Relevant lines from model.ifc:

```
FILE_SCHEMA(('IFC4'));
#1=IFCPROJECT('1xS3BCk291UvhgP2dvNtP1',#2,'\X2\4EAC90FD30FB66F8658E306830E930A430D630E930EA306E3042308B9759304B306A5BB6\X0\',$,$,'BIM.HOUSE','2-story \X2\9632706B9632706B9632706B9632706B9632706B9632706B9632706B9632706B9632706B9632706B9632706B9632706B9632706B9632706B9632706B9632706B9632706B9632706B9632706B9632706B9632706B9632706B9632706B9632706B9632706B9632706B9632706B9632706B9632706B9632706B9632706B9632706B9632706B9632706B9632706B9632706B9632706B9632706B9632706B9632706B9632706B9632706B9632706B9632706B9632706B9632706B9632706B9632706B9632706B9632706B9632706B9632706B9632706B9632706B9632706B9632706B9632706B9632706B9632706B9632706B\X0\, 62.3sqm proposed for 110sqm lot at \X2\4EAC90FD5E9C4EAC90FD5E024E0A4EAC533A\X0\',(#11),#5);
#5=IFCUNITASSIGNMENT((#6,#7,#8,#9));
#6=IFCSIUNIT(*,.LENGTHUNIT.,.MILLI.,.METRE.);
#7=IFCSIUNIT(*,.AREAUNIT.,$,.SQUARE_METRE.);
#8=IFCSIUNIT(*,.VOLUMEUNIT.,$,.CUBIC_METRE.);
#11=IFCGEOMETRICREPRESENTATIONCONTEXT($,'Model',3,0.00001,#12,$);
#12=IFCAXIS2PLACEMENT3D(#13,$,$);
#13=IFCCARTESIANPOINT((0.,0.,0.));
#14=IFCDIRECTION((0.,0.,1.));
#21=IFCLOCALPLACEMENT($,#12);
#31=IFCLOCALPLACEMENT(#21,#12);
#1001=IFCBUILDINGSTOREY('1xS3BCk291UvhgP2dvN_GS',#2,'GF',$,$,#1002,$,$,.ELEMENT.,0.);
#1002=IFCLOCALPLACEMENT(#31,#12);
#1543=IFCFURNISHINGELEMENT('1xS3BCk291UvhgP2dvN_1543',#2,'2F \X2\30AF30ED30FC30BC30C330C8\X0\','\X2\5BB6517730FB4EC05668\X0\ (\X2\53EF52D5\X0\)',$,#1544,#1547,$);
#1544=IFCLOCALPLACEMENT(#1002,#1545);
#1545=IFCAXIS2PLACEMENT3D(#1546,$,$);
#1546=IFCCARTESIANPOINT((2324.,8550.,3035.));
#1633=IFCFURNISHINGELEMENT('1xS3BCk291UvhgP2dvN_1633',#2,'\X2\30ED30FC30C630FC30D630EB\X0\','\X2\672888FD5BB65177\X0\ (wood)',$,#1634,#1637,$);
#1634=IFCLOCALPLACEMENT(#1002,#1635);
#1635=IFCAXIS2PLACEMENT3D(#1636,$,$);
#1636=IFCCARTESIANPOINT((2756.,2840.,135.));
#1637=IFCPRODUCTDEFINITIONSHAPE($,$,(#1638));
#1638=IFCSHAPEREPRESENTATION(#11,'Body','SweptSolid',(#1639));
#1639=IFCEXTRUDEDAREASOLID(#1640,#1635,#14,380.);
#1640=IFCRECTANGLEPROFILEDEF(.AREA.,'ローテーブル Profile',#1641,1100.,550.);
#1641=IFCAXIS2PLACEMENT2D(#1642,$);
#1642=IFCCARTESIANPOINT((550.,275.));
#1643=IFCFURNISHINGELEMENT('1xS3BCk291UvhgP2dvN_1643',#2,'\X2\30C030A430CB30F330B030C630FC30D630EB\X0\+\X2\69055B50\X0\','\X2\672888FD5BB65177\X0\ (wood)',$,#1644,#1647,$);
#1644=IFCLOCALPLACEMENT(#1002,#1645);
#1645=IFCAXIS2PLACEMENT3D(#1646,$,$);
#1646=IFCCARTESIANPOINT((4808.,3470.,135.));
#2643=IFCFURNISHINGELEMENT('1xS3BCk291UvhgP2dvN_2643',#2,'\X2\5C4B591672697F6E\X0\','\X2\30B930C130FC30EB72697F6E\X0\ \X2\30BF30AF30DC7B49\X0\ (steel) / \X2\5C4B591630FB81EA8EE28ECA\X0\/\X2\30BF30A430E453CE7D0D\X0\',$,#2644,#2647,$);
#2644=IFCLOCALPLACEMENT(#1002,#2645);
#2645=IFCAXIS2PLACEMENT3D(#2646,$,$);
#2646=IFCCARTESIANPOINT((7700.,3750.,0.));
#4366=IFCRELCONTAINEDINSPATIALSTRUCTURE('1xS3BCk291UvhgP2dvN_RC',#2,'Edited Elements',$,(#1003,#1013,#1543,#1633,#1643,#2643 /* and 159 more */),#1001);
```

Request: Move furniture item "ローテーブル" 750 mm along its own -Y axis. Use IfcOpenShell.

```python
import ifcopenshell
import ifcopenshell.api.geometry
import ifcopenshell.util.placement
import ifcopenshell.util.unit

model = ifcopenshell.open("model.ifc")
unit_scale = ifcopenshell.util.unit.calculate_unit_scale(model)

item = model.by_guid("1xS3BCk291UvhgP2dvN_1633")
matrix = ifcopenshell.util.placement.get_local_placement(item.ObjectPlacement)
matrix[:3, 3] -= matrix[:3, 1] * 0.75 / unit_scale
ifcopenshell.api.geometry.edit_object_placement(model, product=item, matrix=matrix, is_si=False)

print(ifcopenshell.util.placement.get_local_placement(item.ObjectPlacement).round(3) + 0.0)

model.write("model_v2.ifc")
```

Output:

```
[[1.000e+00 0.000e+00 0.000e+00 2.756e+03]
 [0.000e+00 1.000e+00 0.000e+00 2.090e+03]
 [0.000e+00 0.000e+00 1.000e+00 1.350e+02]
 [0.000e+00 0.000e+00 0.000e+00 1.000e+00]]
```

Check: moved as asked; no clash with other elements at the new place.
